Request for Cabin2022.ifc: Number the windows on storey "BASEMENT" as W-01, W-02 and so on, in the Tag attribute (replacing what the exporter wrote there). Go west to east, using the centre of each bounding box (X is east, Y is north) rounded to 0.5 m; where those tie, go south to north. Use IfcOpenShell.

First a look at what the model holds.

```python
import ifcopenshell
import ifcopenshell.util.element
import ifcopenshell.util.placement

model = ifcopenshell.open("Cabin2022.ifc")
print(model.schema)
storey = next(s for s in model.by_type("IfcBuildingStorey") if s.Name == "BASEMENT")
windows = [e for e in ifcopenshell.util.element.get_decomposition(storey) if e.is_a("IfcWindow")]
for e in sorted(windows, key=lambda e: e.id()):
    origin = ifcopenshell.util.placement.get_local_placement(e.ObjectPlacement)[:3, 3]
    print(e.id(), e.Tag, e.Name, origin.round(2) + 0.0, sep=" | ")
```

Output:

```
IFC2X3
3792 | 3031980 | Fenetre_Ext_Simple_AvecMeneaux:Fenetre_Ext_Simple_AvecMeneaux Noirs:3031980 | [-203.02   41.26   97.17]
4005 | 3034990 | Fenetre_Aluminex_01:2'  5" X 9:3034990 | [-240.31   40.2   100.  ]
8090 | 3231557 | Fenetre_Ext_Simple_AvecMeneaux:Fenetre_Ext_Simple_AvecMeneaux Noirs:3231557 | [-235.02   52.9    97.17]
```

```python
import ifcopenshell
import ifcopenshell.geom
import ifcopenshell.util.element
import ifcopenshell.util.shape

model = ifcopenshell.open("Cabin2022.ifc")
settings = ifcopenshell.geom.settings()
settings.set("use-world-coords", True)


def centre(element):
    shape = ifcopenshell.geom.create_shape(settings, element)
    return ifcopenshell.util.shape.get_bbox_centroid(shape.geometry)


storey = next(s for s in model.by_type("IfcBuildingStorey") if s.Name == "BASEMENT")
windows = [e for e in ifcopenshell.util.element.get_decomposition(storey) if e.is_a("IfcWindow")]

# Insertion points can sit at a corner or the storey origin, so sort by the geometry (in metres).
centres = {e: centre(e) for e in windows}
windows.sort(key=lambda e: (round(centres[e][0] / 0.5), centres[e][1]))

for i, e in enumerate(windows, start=1):
    number = f"W-{i:02d}"
    e.Tag = number
    print(e.id(), number)

model.write("Cabin2022_edited.ifc")
```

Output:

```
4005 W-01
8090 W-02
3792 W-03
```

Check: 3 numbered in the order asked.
